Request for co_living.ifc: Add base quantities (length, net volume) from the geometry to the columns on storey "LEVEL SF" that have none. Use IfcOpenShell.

First a look at what the model holds.

```python
import ifcopenshell
import ifcopenshell.util.element
import ifcopenshell.util.unit

model = ifcopenshell.open("co_living.ifc")
print(model.schema)
for unit_type in ("LENGTHUNIT", "AREAUNIT", "VOLUMEUNIT"):
    print(unit_type, ifcopenshell.util.unit.calculate_unit_scale(model, unit_type))
storey = next(s for s in model.by_type("IfcBuildingStorey") if s.Name == "LEVEL SF")
columns = [e for e in ifcopenshell.util.element.get_decomposition(storey) if e.is_a("IfcColumn")]
for e in sorted(columns, key=lambda e: e.id()):
    print(e.id(), e.is_a(), e.Name, list(ifcopenshell.util.element.get_psets(e, qtos_only=True)), sep=" | ")
```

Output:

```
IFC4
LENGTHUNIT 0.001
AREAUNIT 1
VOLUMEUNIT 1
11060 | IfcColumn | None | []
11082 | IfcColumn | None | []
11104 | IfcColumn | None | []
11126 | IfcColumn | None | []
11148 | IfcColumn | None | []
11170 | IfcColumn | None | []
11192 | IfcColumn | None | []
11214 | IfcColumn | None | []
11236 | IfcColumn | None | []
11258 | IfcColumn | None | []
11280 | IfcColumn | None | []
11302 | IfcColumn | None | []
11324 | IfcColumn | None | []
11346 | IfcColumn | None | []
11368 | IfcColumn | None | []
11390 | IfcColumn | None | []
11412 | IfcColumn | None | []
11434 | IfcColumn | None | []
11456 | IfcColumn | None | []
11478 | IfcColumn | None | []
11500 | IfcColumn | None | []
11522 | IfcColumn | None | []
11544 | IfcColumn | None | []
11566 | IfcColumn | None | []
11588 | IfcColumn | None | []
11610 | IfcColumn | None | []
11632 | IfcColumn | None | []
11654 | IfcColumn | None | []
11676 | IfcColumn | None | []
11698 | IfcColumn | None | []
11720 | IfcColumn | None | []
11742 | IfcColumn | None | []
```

```python
import ifcopenshell
import ifcopenshell.api.pset
import ifcopenshell.geom
import ifcopenshell.util.element
import ifcopenshell.util.shape
import ifcopenshell.util.unit

model = ifcopenshell.open("co_living.ifc")
unit_scale = ifcopenshell.util.unit.calculate_unit_scale(model)
volume_scale = ifcopenshell.util.unit.calculate_unit_scale(model, "VOLUMEUNIT")
settings = ifcopenshell.geom.settings()

storey = next(s for s in model.by_type("IfcBuildingStorey") if s.Name == "LEVEL SF")
columns = [e for e in ifcopenshell.util.element.get_decomposition(storey) if e.is_a("IfcColumn")]

for e in sorted(columns, key=lambda e: e.id()):
    if ifcopenshell.util.element.get_psets(e, qtos_only=True, should_inherit=False):
        continue
    # Geometry comes back in metres, in the element's own axes.
    shape = ifcopenshell.geom.create_shape(settings, e)
    values = {
        "Length": ifcopenshell.util.shape.get_z(shape.geometry) / unit_scale,
        "NetVolume": ifcopenshell.util.shape.get_volume(shape.geometry) / volume_scale,
    }
    qto = ifcopenshell.api.pset.add_qto(model, product=e, name="Qto_ColumnBaseQuantities")
    ifcopenshell.api.pset.edit_qto(model, qto=qto, properties=values)
    print(e.id(), {k: round(v, 3) for k, v in values.items()})

model.write("co_living_rev.ifc")
```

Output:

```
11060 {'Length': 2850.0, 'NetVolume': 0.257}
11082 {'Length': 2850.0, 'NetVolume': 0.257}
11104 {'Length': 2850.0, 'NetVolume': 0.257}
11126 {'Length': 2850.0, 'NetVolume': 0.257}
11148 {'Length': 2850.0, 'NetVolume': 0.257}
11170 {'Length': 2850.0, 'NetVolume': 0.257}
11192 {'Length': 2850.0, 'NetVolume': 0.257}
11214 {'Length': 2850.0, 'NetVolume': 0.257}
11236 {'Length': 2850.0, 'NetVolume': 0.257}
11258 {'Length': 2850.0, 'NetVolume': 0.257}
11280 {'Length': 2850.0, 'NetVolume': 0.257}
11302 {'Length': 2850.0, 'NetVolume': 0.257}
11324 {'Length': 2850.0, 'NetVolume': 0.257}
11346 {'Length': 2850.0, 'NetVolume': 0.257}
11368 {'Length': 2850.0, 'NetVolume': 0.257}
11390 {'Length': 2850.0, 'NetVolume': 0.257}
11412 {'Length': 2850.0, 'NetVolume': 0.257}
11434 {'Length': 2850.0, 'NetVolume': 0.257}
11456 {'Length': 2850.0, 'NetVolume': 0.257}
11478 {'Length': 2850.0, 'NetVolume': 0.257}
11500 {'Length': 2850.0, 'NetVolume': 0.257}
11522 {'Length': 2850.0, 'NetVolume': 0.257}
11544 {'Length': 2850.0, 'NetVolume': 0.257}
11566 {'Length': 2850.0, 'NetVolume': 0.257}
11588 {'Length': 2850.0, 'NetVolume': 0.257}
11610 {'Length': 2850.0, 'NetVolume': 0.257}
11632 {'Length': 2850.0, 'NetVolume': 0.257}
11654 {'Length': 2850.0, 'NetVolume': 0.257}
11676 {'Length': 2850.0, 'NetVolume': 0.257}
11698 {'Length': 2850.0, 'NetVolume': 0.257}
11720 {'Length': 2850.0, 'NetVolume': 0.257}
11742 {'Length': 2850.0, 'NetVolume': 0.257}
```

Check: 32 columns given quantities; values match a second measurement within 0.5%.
